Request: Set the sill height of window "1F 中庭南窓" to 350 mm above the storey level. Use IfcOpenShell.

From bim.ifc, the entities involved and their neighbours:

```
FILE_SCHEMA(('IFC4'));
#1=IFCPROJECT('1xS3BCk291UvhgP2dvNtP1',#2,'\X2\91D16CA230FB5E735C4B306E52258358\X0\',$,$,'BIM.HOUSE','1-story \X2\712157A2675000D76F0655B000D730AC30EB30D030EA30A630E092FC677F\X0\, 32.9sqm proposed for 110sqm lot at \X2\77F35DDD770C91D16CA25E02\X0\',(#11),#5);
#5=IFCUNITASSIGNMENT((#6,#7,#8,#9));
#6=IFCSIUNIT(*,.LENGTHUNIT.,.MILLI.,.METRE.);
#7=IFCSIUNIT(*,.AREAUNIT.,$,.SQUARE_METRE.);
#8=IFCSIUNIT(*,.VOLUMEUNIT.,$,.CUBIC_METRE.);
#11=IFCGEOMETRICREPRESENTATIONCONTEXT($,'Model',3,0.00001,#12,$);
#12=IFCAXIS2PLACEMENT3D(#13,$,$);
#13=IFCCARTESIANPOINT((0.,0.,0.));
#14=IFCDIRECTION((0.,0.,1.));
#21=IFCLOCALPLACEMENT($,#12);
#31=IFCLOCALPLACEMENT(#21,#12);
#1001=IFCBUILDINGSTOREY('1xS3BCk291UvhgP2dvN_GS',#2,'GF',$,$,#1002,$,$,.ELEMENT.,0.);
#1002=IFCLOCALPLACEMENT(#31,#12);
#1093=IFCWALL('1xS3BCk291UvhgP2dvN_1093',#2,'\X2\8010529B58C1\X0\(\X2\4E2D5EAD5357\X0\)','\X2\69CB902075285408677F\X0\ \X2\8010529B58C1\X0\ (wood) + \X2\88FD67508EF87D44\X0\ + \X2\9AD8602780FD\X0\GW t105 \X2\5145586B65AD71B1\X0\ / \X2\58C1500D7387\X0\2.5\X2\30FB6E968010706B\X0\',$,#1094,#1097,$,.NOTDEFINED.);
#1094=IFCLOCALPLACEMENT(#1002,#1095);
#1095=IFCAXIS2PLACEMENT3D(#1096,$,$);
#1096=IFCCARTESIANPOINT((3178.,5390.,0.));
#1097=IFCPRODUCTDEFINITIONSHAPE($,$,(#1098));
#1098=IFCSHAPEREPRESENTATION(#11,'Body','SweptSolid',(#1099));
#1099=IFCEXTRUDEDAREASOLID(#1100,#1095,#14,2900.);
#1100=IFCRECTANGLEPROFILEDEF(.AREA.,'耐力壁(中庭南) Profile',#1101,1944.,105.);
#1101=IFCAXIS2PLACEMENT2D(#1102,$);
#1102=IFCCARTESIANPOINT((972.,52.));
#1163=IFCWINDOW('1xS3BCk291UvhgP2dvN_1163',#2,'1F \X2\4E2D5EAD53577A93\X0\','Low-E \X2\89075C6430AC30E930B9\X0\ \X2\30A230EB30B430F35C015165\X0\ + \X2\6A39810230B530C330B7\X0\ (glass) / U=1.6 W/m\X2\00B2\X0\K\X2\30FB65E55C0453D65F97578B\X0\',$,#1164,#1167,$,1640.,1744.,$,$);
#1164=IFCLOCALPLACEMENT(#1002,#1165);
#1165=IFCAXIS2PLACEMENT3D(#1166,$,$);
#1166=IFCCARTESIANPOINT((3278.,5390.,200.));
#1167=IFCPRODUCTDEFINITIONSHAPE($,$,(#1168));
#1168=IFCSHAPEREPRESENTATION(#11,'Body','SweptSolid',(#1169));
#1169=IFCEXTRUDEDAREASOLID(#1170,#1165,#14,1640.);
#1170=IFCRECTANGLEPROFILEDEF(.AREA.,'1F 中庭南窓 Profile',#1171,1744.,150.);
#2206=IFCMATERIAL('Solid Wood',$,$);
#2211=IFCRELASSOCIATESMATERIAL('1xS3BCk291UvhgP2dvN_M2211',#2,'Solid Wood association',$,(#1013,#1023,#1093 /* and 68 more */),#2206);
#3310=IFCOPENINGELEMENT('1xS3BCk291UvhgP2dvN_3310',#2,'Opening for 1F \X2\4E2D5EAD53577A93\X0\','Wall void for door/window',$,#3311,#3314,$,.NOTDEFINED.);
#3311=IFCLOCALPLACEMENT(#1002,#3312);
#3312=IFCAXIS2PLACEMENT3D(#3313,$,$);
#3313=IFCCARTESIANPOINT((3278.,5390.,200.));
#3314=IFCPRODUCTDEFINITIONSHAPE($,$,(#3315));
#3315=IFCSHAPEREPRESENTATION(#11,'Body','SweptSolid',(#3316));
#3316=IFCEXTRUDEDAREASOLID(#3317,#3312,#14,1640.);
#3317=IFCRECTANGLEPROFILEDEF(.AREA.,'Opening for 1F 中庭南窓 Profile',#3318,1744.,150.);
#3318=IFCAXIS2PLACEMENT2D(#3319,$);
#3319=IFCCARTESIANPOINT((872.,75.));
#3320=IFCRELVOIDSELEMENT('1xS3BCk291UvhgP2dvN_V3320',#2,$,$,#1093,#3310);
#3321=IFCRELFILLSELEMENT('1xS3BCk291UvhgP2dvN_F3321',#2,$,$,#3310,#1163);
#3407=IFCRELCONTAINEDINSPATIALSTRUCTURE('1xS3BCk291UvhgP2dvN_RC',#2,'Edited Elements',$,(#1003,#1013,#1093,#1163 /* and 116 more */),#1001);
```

```python
import numpy as np
import ifcopenshell
import ifcopenshell.api.geometry
import ifcopenshell.geom
import ifcopenshell.util.element
import ifcopenshell.util.placement
import ifcopenshell.util.shape
import ifcopenshell.util.unit

model = ifcopenshell.open("bim.ifc")
unit_scale = ifcopenshell.util.unit.calculate_unit_scale(model)

window = model.by_guid("1xS3BCk291UvhgP2dvN_1163")
opening = window.FillsVoids[0].RelatingOpeningElement
storey = ifcopenshell.util.element.get_container(window, ifc_class="IfcBuildingStorey")
level = ifcopenshell.util.placement.get_local_placement(storey.ObjectPlacement)[2, 3]

# The opening's origin need not be at the sill, so measure its lowest point.
shape = ifcopenshell.geom.create_shape(ifcopenshell.geom.settings(), opening)
bottom = ifcopenshell.util.shape.get_shape_bottom_elevation(shape, shape.geometry) / unit_scale
dz = level + 0.35 / unit_scale - bottom

shift = np.array([0.0, 0.0, dz])
# The window is not placed relative to its opening, so move both.
for product in (opening, window):
    matrix = ifcopenshell.util.placement.get_local_placement(product.ObjectPlacement)
    matrix[:3, 3] += shift
    ifcopenshell.api.geometry.edit_object_placement(model, product=product, matrix=matrix, is_si=False)

print(f"moved by {dz * unit_scale:+.3f} m")

model.write("bim_edited.ifc")
```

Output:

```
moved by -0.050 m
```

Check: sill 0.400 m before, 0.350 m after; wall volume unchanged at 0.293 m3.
